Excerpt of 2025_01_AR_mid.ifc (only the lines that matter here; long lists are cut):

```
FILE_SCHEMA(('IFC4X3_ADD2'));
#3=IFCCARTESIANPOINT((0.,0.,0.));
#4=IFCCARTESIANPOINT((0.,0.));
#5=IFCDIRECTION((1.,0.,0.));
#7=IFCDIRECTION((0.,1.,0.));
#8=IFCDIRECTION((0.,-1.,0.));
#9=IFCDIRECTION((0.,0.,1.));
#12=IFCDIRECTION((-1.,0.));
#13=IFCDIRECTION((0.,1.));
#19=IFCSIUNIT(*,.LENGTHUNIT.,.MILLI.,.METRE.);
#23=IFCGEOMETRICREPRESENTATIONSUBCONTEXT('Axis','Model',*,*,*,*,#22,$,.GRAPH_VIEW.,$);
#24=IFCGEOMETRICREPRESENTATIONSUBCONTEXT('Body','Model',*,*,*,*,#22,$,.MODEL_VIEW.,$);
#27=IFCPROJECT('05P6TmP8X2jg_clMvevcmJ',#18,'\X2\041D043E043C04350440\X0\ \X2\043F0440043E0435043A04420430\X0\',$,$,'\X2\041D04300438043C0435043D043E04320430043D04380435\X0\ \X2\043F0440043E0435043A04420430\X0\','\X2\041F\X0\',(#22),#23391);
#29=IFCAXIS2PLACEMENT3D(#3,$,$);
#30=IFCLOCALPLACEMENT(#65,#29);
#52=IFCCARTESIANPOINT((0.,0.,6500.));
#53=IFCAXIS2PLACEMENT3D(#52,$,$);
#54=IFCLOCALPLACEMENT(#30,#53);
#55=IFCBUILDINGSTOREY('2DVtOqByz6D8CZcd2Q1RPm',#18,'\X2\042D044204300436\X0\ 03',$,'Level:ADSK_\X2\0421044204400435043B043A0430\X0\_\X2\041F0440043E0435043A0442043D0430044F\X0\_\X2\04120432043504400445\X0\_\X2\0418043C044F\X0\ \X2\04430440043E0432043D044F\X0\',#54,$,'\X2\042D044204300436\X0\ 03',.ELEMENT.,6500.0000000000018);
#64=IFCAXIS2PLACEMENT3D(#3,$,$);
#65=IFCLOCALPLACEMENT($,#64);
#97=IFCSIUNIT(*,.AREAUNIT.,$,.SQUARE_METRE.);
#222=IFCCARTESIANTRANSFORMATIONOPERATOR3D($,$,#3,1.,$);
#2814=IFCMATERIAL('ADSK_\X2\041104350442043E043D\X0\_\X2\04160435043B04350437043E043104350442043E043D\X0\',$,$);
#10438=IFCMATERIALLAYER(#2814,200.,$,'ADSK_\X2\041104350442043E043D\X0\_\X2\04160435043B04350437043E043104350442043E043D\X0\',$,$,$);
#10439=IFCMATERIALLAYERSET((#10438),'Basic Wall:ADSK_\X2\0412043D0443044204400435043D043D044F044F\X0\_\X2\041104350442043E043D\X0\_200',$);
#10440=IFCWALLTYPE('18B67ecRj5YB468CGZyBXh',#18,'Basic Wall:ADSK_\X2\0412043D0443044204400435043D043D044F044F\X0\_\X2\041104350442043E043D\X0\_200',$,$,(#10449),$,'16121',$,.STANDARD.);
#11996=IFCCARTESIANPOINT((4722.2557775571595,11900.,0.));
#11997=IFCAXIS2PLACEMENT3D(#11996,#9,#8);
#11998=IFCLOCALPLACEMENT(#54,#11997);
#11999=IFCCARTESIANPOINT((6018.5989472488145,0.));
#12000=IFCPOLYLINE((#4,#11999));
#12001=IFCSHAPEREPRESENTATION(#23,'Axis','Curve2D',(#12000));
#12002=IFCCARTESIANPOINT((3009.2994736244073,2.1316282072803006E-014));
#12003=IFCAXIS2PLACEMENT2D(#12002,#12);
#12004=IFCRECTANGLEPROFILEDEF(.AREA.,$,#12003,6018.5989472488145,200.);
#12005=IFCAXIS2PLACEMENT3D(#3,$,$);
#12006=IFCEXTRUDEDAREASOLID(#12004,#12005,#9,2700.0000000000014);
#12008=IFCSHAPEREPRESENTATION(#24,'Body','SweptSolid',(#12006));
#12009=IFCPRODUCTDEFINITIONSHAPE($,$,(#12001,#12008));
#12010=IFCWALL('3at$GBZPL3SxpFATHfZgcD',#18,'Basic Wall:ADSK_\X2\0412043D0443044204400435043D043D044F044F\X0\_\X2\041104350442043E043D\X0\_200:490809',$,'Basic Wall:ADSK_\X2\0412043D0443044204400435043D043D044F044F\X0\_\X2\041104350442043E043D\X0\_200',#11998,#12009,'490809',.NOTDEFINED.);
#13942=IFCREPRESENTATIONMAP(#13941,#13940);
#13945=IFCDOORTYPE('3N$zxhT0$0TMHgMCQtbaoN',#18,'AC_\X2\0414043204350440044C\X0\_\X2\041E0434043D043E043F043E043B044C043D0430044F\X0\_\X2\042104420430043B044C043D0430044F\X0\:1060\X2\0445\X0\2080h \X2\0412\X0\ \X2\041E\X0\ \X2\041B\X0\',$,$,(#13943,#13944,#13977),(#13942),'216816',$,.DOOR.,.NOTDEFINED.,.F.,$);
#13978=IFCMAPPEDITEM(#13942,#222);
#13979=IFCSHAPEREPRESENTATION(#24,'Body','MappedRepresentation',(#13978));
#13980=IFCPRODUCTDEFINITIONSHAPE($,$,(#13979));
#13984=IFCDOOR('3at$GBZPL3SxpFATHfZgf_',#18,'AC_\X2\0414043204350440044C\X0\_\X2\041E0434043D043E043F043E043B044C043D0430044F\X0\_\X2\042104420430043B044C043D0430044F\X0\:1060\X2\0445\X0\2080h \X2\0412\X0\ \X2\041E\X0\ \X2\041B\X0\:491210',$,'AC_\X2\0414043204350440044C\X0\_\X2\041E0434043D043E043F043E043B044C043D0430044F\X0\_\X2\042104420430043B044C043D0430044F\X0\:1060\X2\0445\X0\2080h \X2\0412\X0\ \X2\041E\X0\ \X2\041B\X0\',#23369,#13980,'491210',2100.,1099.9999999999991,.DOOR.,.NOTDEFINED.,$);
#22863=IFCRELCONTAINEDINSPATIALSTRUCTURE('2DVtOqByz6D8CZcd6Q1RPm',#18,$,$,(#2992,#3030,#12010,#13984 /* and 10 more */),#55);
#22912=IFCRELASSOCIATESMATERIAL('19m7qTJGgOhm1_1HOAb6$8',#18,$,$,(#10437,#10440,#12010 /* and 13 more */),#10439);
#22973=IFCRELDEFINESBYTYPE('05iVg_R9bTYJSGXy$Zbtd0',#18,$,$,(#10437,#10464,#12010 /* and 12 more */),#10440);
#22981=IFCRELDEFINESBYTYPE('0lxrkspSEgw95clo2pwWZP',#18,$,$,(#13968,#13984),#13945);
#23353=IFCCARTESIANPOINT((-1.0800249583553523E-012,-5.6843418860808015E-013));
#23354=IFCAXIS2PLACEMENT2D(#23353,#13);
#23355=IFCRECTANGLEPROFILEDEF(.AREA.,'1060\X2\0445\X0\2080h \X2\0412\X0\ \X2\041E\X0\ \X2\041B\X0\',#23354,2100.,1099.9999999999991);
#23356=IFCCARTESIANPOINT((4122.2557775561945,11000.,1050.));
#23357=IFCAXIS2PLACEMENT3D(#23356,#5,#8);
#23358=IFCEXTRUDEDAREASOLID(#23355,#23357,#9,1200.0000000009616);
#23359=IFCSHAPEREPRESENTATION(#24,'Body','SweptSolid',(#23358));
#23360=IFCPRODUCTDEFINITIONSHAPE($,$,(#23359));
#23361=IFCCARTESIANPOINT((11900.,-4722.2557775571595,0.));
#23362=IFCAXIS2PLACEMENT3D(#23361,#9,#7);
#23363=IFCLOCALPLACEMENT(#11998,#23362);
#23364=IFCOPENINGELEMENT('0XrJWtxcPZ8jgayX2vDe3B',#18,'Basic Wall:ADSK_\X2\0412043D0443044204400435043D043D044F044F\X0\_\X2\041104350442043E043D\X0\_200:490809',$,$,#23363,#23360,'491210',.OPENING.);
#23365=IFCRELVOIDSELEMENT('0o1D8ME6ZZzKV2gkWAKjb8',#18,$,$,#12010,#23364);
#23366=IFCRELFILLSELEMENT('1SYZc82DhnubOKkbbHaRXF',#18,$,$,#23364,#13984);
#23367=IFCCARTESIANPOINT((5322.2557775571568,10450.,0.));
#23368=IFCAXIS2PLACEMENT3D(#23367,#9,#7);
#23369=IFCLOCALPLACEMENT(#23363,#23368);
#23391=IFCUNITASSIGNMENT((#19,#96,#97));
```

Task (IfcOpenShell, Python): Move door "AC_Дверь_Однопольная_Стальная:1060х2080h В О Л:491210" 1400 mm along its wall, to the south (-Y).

```python
import ifcopenshell
import ifcopenshell.api.geometry
import ifcopenshell.util.placement
import ifcopenshell.util.unit

model = ifcopenshell.open("2025_01_AR_mid.ifc")
unit_scale = ifcopenshell.util.unit.calculate_unit_scale(model)

door = model.by_id(13984)
opening = door.FillsVoids[0].RelatingOpeningElement
wall = opening.VoidsElements[0].RelatingBuildingElement

wall_matrix = ifcopenshell.util.placement.get_local_placement(wall.ObjectPlacement)
shift = wall_matrix[:3, 0] * 1.4 / unit_scale
before = ifcopenshell.util.placement.get_local_placement(door.ObjectPlacement)[:3, 3].copy()

# The door is placed relative to its opening, so it follows when the opening moves.
matrix = ifcopenshell.util.placement.get_local_placement(opening.ObjectPlacement)
matrix[:3, 3] += shift
ifcopenshell.api.geometry.edit_object_placement(
    model, product=opening, matrix=matrix, is_si=False, should_transform_children=True
)

after = ifcopenshell.util.placement.get_local_placement(door.ObjectPlacement)[:3, 3]
print("door moved by", (after - before).round(3) + 0.0)

model.write("2025_01_AR_mid-out.ifc")
```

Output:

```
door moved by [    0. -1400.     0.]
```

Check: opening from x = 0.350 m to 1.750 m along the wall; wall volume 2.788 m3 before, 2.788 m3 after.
